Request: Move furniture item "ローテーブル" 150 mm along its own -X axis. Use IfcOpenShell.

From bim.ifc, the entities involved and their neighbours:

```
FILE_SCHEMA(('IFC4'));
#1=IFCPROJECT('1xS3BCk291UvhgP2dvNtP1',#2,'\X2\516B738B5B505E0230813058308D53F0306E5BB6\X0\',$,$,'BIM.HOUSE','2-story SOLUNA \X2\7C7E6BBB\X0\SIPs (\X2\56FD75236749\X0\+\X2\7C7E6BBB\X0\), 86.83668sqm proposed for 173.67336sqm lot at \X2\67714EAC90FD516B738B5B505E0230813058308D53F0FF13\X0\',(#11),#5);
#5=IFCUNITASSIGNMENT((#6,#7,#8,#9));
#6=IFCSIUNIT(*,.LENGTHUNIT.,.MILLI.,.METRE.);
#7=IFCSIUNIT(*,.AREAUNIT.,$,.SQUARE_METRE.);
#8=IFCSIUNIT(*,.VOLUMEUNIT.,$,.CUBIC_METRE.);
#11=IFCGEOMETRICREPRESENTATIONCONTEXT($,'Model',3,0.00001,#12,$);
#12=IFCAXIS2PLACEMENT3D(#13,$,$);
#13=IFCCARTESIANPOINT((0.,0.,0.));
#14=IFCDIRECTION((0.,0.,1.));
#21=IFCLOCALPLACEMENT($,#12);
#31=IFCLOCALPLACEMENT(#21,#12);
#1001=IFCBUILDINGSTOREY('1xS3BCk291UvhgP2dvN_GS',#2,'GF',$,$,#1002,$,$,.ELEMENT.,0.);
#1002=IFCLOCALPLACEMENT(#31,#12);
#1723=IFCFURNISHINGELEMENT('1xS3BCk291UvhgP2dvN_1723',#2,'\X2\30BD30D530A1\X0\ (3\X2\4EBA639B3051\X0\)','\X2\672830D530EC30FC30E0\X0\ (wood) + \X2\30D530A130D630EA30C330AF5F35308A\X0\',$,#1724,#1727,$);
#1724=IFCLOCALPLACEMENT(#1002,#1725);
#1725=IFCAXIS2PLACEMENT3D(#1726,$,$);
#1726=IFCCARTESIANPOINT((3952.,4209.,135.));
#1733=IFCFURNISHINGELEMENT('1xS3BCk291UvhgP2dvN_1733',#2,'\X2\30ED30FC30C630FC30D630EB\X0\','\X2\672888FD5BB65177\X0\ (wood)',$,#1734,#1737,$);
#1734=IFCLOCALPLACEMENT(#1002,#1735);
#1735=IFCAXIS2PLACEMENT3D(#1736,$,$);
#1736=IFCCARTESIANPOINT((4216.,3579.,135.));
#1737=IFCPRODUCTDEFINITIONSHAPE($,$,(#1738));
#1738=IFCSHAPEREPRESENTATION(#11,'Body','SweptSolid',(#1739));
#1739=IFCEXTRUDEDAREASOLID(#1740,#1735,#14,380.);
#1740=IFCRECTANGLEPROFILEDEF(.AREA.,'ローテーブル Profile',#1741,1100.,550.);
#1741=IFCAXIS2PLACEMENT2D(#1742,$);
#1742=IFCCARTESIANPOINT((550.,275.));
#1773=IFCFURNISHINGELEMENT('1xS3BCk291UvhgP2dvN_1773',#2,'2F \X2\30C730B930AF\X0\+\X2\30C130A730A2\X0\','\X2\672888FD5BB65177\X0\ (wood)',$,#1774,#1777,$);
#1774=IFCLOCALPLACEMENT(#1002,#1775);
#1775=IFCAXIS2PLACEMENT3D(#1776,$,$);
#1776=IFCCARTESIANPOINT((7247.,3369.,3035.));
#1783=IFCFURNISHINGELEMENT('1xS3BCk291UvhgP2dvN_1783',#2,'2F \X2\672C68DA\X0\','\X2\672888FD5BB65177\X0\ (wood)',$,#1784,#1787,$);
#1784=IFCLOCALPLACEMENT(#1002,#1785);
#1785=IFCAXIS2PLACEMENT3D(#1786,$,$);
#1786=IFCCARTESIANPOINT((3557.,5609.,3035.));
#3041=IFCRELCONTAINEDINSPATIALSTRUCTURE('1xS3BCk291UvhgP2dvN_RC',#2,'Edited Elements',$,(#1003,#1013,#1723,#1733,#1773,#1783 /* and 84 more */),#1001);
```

```python
import ifcopenshell
import ifcopenshell.api.geometry
import ifcopenshell.util.placement

model = ifcopenshell.open("bim.ifc")

item = model.by_id(1733)
matrix = ifcopenshell.util.placement.get_local_placement(item.ObjectPlacement)
matrix[:3, 3] -= matrix[:3, 0] * 150.0
ifcopenshell.api.geometry.edit_object_placement(model, product=item, matrix=matrix, is_si=False)

print(ifcopenshell.util.placement.get_local_placement(item.ObjectPlacement).round(3) + 0.0)

model.write("bim-out.ifc")
```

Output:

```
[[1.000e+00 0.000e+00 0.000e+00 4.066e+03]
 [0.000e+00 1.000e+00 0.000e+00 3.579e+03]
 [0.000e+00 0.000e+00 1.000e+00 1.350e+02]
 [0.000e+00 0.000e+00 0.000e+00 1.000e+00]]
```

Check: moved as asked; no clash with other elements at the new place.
